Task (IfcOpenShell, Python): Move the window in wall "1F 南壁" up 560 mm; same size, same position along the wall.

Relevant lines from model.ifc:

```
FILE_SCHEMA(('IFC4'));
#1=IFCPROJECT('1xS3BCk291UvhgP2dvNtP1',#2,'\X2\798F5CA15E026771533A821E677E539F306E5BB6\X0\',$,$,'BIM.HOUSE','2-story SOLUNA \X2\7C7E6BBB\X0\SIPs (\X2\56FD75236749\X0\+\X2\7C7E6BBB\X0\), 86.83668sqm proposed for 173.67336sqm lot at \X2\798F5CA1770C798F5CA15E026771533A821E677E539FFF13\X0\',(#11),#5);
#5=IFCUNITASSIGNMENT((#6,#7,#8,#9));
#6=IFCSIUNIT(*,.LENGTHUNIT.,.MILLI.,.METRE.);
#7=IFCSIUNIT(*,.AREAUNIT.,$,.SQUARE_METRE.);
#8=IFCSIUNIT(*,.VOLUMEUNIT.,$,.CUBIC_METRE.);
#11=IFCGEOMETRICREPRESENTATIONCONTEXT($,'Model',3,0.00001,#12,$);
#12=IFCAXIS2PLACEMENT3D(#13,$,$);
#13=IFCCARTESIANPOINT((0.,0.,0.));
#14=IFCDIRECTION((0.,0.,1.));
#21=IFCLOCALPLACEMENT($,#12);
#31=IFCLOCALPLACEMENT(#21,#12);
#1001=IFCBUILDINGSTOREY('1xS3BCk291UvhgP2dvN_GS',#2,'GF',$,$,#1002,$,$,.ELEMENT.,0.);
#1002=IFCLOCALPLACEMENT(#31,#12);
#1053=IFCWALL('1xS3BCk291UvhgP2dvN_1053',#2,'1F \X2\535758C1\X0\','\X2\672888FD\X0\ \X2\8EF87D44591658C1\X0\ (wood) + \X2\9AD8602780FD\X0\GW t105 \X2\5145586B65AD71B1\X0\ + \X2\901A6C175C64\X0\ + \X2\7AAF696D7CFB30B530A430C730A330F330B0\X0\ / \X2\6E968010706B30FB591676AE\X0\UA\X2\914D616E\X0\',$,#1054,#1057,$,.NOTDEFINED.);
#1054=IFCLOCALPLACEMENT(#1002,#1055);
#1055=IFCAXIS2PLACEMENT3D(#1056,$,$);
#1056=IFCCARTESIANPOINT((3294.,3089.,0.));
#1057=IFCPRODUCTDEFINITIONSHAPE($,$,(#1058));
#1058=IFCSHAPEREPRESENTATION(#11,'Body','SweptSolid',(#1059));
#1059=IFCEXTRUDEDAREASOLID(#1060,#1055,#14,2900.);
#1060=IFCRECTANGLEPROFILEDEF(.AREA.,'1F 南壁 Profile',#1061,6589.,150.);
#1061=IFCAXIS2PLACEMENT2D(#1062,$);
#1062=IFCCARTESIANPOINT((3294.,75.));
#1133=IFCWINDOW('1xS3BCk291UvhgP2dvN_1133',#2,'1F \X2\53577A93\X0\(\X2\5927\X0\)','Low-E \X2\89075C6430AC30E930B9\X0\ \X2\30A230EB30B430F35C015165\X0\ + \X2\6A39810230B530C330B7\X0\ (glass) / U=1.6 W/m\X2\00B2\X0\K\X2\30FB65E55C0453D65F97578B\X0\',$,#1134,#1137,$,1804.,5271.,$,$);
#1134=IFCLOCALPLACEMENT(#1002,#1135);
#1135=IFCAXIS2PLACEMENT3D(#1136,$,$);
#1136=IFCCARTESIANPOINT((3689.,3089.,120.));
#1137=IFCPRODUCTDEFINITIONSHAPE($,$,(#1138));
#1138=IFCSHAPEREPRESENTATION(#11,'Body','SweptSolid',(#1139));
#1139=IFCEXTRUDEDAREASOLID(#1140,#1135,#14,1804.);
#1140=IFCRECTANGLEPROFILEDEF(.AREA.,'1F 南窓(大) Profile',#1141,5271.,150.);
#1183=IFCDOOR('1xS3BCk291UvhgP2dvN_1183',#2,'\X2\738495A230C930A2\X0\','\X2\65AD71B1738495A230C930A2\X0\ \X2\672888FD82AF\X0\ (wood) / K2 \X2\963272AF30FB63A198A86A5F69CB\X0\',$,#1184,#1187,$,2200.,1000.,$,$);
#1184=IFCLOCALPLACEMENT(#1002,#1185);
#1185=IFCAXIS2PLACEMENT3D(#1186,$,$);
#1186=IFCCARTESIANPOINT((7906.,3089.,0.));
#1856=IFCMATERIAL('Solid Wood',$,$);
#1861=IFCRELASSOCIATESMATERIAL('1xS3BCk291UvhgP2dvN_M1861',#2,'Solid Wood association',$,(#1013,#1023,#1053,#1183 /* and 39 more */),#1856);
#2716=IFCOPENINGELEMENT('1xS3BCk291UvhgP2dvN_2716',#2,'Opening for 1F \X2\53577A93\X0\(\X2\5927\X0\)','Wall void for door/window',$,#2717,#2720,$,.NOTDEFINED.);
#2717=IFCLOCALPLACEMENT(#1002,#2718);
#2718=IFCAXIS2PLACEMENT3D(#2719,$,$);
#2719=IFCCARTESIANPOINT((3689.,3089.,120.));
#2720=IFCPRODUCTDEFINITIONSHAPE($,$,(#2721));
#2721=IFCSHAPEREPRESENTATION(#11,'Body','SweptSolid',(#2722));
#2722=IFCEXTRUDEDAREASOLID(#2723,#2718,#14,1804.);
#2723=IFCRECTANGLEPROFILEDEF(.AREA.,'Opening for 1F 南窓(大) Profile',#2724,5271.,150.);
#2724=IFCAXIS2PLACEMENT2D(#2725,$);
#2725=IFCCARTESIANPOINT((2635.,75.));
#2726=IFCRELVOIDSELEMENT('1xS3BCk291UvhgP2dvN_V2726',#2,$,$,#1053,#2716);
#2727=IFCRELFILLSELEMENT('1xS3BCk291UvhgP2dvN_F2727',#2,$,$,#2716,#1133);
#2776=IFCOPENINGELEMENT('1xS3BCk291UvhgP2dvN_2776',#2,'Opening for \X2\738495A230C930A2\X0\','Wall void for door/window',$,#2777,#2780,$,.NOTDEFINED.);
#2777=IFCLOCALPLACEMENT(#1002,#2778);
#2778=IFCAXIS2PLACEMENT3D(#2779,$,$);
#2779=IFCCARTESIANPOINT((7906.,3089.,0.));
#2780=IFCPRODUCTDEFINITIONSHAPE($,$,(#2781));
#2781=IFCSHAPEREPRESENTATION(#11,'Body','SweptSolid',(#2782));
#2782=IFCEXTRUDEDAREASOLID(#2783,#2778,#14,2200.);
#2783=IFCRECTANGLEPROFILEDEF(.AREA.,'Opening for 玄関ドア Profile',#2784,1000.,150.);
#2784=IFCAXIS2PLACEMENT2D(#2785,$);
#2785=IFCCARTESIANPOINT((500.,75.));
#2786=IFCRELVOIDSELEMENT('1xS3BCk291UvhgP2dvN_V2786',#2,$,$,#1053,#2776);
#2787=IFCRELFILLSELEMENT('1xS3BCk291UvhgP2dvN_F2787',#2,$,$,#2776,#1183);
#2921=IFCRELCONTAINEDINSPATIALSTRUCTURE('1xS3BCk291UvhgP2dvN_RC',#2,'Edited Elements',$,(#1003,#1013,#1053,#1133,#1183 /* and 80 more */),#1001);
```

```python
import numpy as np
import ifcopenshell
import ifcopenshell.api.geometry
import ifcopenshell.util.placement
import ifcopenshell.util.unit

model = ifcopenshell.open("model.ifc")
unit_scale = ifcopenshell.util.unit.calculate_unit_scale(model)

window = model.by_guid("1xS3BCk291UvhgP2dvN_1133")
opening = window.FillsVoids[0].RelatingOpeningElement
dz = 0.56 / unit_scale

shift = np.array([0.0, 0.0, dz])
# The window is not placed relative to its opening, so move both.
for product in (opening, window):
    matrix = ifcopenshell.util.placement.get_local_placement(product.ObjectPlacement)
    matrix[:3, 3] += shift
    ifcopenshell.api.geometry.edit_object_placement(model, product=product, matrix=matrix, is_si=False)

print(f"moved by {dz * unit_scale:+.3f} m")

model.write("model-out.ifc")
```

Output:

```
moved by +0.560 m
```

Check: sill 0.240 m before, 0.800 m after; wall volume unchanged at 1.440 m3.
